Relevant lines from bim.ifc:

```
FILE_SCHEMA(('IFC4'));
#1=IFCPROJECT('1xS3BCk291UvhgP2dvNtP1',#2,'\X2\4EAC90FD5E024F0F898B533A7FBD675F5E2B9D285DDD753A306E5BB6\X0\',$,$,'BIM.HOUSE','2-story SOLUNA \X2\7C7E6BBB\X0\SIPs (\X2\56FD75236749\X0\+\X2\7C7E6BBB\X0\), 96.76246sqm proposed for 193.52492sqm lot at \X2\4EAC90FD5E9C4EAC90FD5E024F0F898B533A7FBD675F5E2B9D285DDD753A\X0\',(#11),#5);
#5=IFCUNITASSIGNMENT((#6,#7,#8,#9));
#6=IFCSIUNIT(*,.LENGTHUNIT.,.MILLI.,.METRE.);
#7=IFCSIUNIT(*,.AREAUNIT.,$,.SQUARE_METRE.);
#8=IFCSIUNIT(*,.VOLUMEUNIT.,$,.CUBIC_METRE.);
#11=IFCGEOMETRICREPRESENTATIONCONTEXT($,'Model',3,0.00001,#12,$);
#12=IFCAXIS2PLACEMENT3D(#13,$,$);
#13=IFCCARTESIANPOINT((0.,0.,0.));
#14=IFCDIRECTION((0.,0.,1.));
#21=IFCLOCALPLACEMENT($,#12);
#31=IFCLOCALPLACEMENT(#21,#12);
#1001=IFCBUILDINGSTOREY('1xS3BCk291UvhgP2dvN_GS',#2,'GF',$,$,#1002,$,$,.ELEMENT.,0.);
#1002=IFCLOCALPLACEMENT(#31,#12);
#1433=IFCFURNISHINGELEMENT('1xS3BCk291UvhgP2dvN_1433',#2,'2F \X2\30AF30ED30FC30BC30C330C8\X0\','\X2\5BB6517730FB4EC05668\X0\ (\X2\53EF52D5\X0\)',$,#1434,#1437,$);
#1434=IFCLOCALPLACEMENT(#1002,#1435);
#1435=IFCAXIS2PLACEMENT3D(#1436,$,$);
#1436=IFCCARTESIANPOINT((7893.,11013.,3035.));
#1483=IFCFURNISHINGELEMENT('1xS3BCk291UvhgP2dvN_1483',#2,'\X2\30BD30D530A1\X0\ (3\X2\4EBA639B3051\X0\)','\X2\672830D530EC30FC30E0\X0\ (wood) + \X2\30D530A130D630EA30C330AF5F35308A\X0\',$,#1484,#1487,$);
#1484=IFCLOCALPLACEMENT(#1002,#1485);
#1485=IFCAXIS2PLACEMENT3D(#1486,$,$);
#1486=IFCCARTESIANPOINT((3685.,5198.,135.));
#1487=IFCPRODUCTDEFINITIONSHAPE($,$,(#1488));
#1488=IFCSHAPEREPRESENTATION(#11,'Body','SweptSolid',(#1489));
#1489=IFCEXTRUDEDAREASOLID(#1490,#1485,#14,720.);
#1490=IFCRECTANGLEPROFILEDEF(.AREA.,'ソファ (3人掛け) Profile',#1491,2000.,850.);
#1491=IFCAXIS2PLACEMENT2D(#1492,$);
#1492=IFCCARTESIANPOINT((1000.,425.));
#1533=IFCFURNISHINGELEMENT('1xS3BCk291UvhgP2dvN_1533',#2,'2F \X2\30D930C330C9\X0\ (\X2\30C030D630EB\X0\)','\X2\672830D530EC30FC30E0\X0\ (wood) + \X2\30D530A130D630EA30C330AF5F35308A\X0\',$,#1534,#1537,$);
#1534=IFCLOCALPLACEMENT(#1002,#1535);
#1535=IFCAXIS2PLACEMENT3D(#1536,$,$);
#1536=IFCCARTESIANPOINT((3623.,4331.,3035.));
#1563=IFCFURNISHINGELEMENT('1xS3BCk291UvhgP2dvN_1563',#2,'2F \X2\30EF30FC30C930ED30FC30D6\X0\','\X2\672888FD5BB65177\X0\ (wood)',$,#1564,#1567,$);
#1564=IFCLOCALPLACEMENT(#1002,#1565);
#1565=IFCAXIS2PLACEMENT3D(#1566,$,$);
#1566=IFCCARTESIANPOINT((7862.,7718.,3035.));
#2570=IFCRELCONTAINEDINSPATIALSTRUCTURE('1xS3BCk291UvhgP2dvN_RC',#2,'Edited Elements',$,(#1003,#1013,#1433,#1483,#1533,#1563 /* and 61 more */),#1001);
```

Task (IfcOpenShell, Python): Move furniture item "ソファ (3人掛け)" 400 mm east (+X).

```python
import ifcopenshell
import ifcopenshell.api.geometry
import ifcopenshell.util.placement
import ifcopenshell.util.unit

model = ifcopenshell.open("bim.ifc")
unit_scale = ifcopenshell.util.unit.calculate_unit_scale(model)

item = model.by_id(1483)
matrix = ifcopenshell.util.placement.get_local_placement(item.ObjectPlacement)
matrix[0, 3] += 0.4 / unit_scale
ifcopenshell.api.geometry.edit_object_placement(model, product=item, matrix=matrix, is_si=False)

print(ifcopenshell.util.placement.get_local_placement(item.ObjectPlacement).round(3) + 0.0)

model.write("bim_updated.ifc")
```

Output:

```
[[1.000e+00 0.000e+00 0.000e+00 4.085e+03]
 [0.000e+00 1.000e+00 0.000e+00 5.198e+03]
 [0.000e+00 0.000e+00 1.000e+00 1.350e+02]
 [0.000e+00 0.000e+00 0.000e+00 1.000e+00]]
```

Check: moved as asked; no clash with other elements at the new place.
